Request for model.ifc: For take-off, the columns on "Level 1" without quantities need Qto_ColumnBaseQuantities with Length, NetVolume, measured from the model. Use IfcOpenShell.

First a look at what the model holds.

```python
import ifcopenshell
import ifcopenshell.util.element
import ifcopenshell.util.unit

model = ifcopenshell.open("model.ifc")
print(model.schema)
for unit_type in ("LENGTHUNIT", "AREAUNIT", "VOLUMEUNIT"):
    print(unit_type, ifcopenshell.util.unit.calculate_unit_scale(model, unit_type))
storey = next(s for s in model.by_type("IfcBuildingStorey") if s.Name == "Level 1")
columns = [e for e in ifcopenshell.util.element.get_decomposition(storey) if e.is_a("IfcColumn")]
for e in sorted(columns, key=lambda e: e.id()):
    print(e.id(), e.is_a(), e.Name, list(ifcopenshell.util.element.get_psets(e, qtos_only=True)), sep=" | ")
```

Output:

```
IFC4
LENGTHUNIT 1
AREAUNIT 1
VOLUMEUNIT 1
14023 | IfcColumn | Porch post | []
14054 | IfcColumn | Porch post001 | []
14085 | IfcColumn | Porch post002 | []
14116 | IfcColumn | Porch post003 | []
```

```python
import ifcopenshell
import ifcopenshell.api.pset
import ifcopenshell.geom
import ifcopenshell.util.element
import ifcopenshell.util.shape
import ifcopenshell.util.unit

model = ifcopenshell.open("model.ifc")
unit_scale = ifcopenshell.util.unit.calculate_unit_scale(model)
volume_scale = ifcopenshell.util.unit.calculate_unit_scale(model, "VOLUMEUNIT")
settings = ifcopenshell.geom.settings()

storey = next(s for s in model.by_type("IfcBuildingStorey") if s.Name == "Level 1")
columns = [e for e in ifcopenshell.util.element.get_decomposition(storey) if e.is_a("IfcColumn")]

for e in sorted(columns, key=lambda e: e.id()):
    if ifcopenshell.util.element.get_psets(e, qtos_only=True, should_inherit=False):
        continue
    # Geometry comes back in metres, in the element's own axes.
    shape = ifcopenshell.geom.create_shape(settings, e)
    values = {
        "Length": ifcopenshell.util.shape.get_z(shape.geometry) / unit_scale,
        "NetVolume": ifcopenshell.util.shape.get_volume(shape.geometry) / volume_scale,
    }
    qto = ifcopenshell.api.pset.add_qto(model, product=e, name="Qto_ColumnBaseQuantities")
    ifcopenshell.api.pset.edit_qto(model, qto=qto, properties=values)
    print(e.id(), {k: round(v, 3) for k, v in values.items()})

model.write("model-out.ifc")
```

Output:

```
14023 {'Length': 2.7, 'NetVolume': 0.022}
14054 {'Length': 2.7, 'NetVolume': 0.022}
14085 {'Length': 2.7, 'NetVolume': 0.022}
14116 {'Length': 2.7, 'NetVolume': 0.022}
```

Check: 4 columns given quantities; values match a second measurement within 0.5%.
